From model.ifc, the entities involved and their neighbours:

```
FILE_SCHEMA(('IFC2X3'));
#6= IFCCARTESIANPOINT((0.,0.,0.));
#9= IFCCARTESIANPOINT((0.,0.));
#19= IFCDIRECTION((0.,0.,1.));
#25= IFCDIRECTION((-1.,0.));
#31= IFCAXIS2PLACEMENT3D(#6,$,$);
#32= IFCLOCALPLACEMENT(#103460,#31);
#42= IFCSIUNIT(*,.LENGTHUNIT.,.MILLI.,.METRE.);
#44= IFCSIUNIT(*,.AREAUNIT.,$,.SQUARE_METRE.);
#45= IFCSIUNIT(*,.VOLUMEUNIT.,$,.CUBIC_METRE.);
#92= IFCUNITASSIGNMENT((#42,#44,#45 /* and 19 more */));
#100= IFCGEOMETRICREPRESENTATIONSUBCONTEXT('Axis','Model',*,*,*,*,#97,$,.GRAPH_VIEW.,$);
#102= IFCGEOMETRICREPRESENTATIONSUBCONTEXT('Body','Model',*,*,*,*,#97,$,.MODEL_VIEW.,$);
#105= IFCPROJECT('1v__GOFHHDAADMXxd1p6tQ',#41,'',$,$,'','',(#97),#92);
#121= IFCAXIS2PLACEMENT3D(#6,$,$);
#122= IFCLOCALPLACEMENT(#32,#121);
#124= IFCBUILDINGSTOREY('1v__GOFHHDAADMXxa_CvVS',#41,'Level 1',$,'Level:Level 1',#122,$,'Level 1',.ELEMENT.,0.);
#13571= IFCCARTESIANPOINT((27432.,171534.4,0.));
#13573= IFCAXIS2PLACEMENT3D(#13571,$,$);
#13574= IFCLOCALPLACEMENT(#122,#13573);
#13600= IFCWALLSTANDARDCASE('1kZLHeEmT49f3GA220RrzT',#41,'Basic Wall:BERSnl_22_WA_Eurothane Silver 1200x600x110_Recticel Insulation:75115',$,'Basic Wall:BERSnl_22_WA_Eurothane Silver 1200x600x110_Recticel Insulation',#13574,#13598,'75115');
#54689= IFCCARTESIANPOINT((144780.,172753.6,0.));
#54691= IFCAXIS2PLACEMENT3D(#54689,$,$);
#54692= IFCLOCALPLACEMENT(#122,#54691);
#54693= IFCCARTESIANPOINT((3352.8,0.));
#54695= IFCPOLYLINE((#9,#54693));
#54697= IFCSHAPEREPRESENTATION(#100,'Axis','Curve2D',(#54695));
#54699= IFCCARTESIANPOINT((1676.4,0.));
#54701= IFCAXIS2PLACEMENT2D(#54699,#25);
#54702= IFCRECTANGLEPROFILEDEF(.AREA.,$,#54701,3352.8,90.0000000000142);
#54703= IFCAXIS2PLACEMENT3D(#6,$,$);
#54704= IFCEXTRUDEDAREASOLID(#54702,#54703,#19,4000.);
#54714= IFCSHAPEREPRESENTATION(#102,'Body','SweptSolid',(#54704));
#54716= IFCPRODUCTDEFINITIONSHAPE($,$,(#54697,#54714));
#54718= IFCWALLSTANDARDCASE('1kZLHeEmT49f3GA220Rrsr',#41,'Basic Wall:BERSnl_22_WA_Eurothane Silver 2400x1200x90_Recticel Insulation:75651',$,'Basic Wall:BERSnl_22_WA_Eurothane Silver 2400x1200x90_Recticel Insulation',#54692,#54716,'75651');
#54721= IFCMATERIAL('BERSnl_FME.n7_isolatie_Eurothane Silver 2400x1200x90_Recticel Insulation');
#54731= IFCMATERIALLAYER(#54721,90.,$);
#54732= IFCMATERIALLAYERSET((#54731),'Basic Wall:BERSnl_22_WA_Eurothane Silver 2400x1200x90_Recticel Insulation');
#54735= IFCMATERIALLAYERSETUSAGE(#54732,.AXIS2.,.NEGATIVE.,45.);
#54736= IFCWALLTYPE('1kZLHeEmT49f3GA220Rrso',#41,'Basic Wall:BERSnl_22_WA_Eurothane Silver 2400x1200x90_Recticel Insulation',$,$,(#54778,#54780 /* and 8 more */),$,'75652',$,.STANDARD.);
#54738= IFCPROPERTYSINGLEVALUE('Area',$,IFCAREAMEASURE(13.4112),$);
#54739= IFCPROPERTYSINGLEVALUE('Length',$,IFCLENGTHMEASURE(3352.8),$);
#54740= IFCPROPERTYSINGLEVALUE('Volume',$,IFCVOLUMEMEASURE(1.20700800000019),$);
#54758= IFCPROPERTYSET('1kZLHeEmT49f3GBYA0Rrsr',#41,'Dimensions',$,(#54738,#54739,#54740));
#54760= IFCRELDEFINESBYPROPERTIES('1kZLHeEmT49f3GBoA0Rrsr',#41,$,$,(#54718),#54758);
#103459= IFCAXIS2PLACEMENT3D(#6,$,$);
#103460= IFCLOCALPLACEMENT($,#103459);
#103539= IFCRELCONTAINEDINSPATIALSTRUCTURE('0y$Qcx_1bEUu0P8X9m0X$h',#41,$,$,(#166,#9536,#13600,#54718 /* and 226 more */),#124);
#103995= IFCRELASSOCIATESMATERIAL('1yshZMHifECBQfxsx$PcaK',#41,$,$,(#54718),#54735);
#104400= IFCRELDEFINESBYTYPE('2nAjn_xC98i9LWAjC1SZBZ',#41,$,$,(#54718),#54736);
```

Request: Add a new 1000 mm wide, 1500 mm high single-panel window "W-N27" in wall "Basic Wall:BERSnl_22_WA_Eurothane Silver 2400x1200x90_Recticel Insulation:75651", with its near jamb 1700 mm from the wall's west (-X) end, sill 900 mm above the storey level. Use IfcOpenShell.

```python
import numpy as np
import ifcopenshell
import ifcopenshell.api.feature
import ifcopenshell.api.geometry
import ifcopenshell.api.pset
import ifcopenshell.api.root
import ifcopenshell.api.spatial
import ifcopenshell.api.type
import ifcopenshell.geom
import ifcopenshell.util.element
import ifcopenshell.util.placement
import ifcopenshell.util.representation
import ifcopenshell.util.shape
import ifcopenshell.util.unit

model = ifcopenshell.open("model.ifc")
unit_scale = ifcopenshell.util.unit.calculate_unit_scale(model)
area_scale = ifcopenshell.util.unit.calculate_unit_scale(model, "AREAUNIT")
volume_scale = ifcopenshell.util.unit.calculate_unit_scale(model, "VOLUMEUNIT")
settings = ifcopenshell.geom.settings()


def volume(element):
    """Net volume in cubic metres, openings subtracted."""
    shape = ifcopenshell.geom.create_shape(settings, element)
    return ifcopenshell.util.shape.get_volume(shape.geometry)


wall = model.by_guid("1kZLHeEmT49f3GA220Rrsr")
storey = ifcopenshell.util.element.get_container(wall, ifc_class="IfcBuildingStorey")
context = ifcopenshell.util.representation.get_context(model, "Model", "Body", "MODEL_VIEW")
before = volume(wall)

width, height, from_end, sill = 1, 1.5, 1.7, 0.9  # metres

# The wall runs along its own X axis, and the end named is its -X end.
wall_shape = ifcopenshell.geom.create_shape(settings, wall)
x, y, z = ifcopenshell.util.shape.get_vertices(wall_shape.geometry).T
start = x.min() + from_end
face, thickness = float(y.min()), float(y.max() - y.min())
wall_matrix = ifcopenshell.util.placement.get_local_placement(wall.ObjectPlacement)
level = ifcopenshell.util.placement.get_local_placement(storey.ObjectPlacement)[2, 3]


def in_wall(x, y):
    """Placement at x, y metres in the wall's axes, at sill height."""
    matrix = wall_matrix.copy()
    matrix[:, 3] = wall_matrix @ np.array([x / unit_scale, y / unit_scale, 0.0, 1.0])
    matrix[2, 3] = level + sill / unit_scale
    return matrix


# Opening: a box that overshoots both wall faces by 50 mm.
opening = ifcopenshell.api.root.create_entity(model, ifc_class="IfcOpeningElement")
box = ifcopenshell.api.geometry.add_wall_representation(
    model, context=context, length=width, height=height, thickness=thickness + 0.1
)
ifcopenshell.api.geometry.assign_representation(model, product=opening, representation=box)
ifcopenshell.api.geometry.edit_object_placement(model, product=opening, matrix=in_wall(start, face - 0.05), is_si=False)
ifcopenshell.api.feature.add_feature(model, feature=opening, element=wall)

window = ifcopenshell.api.root.create_entity(model, ifc_class="IfcWindow", name="W-N27")
window.OverallWidth, window.OverallHeight = width / unit_scale, height / unit_scale
body = ifcopenshell.api.geometry.add_window_representation(
    model,
    context=context,
    overall_width=window.OverallWidth,
    overall_height=window.OverallHeight,
    partition_type="SINGLE_PANEL",
)
ifcopenshell.api.geometry.assign_representation(model, product=window, representation=body)
ifcopenshell.api.spatial.assign_container(model, products=[window], relating_structure=storey)
fills = ifcopenshell.api.feature.add_filling(model, opening=opening, element=window)
fills.OwnerHistory = window.OwnerHistory  # required in IFC2X3

# IFC2X3 keeps the operation on the window style.
style = ifcopenshell.api.root.create_entity(model, ifc_class="IfcWindowStyle", name="W-N27")
style.OperationType, style.ConstructionType = "SINGLE_PANEL", "NOTDEFINED"
style.ParameterTakesPrecedence = style.Sizeable = False
ifcopenshell.api.type.assign_type(model, related_objects=[window], relating_type=style)

# Centre the window in the wall's thickness.
ifcopenshell.api.geometry.edit_object_placement(model, product=window, matrix=in_wall(start, face), is_si=False)
window_shape = ifcopenshell.geom.create_shape(settings, window)
depth = ifcopenshell.util.shape.get_vertices(window_shape.geometry)[:, 1]
offset = face + thickness / 2 - (depth.min() + depth.max()) / 2
ifcopenshell.api.geometry.edit_object_placement(model, product=window, matrix=in_wall(start, offset), is_si=False)

after = volume(wall)

# Update the wall's stored quantities.
pset = model.by_id(ifcopenshell.util.element.get_pset(wall, "Dimensions", should_inherit=False)["id"])
ifcopenshell.api.pset.edit_pset(model, pset=pset, properties={
    "Area": model.create_entity("IfcAreaMeasure", after / thickness / area_scale),
    "Volume": model.create_entity("IfcVolumeMeasure", after / volume_scale),
})

print(f"wall volume {before:.3f} -> {after:.3f} m3")

model.write("model-out.ifc")
```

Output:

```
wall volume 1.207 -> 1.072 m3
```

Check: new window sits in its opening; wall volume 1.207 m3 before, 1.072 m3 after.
